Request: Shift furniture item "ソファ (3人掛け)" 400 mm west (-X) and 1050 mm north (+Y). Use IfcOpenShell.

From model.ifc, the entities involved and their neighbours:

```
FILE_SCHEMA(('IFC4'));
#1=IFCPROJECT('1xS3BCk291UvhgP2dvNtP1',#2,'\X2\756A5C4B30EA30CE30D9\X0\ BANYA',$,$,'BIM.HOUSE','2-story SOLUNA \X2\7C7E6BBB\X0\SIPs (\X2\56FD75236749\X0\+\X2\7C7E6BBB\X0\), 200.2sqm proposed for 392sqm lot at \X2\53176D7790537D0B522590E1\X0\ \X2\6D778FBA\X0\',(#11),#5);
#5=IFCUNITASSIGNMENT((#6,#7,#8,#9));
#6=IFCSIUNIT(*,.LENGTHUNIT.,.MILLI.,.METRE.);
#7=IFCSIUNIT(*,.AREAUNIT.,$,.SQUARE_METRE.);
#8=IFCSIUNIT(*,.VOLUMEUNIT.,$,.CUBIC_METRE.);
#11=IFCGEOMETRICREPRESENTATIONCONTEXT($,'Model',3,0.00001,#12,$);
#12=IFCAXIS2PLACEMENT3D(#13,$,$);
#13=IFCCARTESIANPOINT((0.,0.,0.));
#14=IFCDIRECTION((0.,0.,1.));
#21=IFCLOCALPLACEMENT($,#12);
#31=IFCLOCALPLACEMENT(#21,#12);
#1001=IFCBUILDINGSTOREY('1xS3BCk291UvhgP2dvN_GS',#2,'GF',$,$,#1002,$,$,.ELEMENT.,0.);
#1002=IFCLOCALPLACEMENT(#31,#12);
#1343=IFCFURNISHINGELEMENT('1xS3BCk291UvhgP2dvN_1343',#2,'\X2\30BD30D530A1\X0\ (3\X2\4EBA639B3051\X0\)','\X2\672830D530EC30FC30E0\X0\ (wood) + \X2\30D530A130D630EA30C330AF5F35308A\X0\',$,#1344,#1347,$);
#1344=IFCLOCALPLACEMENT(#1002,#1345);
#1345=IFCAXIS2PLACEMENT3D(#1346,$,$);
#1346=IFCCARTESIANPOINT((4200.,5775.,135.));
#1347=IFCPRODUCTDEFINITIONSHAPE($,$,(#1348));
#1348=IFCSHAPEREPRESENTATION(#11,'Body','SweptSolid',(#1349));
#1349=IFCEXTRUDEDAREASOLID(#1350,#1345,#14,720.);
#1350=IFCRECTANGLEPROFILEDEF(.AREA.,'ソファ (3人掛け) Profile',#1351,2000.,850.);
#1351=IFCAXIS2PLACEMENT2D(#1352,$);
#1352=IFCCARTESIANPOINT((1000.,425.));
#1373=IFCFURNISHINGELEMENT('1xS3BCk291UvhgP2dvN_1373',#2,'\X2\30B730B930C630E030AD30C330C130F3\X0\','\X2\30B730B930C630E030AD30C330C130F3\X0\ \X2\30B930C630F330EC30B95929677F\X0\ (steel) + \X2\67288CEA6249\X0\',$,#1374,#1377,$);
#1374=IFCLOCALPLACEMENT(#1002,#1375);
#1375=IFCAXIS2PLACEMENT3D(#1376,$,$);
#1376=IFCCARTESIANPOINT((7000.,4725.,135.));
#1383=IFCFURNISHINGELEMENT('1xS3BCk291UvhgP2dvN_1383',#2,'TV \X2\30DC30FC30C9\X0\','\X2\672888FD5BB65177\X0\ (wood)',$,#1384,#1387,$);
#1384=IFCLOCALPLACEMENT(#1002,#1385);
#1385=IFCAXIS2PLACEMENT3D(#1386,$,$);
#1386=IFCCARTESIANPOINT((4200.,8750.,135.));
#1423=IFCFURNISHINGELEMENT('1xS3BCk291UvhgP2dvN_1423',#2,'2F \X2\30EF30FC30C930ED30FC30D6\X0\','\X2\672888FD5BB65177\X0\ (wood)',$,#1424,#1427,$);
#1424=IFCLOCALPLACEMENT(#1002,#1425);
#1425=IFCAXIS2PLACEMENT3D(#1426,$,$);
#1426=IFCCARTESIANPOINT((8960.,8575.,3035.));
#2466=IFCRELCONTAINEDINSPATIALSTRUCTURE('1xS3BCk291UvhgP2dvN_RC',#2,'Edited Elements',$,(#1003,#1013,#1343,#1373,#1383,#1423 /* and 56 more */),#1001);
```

```python
import ifcopenshell
import ifcopenshell.api.geometry
import ifcopenshell.util.placement
import ifcopenshell.util.unit

model = ifcopenshell.open("model.ifc")
unit_scale = ifcopenshell.util.unit.calculate_unit_scale(model)

item = model.by_id(1343)
matrix = ifcopenshell.util.placement.get_local_placement(item.ObjectPlacement)
matrix[0, 3] -= 0.4 / unit_scale
matrix[1, 3] += 1.05 / unit_scale
ifcopenshell.api.geometry.edit_object_placement(model, product=item, matrix=matrix, is_si=False)

print(ifcopenshell.util.placement.get_local_placement(item.ObjectPlacement).round(3) + 0.0)

model.write("model_v2.ifc")
```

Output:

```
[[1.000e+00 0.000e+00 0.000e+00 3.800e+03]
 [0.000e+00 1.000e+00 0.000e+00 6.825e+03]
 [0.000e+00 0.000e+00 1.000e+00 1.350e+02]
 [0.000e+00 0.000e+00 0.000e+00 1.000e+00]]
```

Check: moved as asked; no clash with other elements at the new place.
